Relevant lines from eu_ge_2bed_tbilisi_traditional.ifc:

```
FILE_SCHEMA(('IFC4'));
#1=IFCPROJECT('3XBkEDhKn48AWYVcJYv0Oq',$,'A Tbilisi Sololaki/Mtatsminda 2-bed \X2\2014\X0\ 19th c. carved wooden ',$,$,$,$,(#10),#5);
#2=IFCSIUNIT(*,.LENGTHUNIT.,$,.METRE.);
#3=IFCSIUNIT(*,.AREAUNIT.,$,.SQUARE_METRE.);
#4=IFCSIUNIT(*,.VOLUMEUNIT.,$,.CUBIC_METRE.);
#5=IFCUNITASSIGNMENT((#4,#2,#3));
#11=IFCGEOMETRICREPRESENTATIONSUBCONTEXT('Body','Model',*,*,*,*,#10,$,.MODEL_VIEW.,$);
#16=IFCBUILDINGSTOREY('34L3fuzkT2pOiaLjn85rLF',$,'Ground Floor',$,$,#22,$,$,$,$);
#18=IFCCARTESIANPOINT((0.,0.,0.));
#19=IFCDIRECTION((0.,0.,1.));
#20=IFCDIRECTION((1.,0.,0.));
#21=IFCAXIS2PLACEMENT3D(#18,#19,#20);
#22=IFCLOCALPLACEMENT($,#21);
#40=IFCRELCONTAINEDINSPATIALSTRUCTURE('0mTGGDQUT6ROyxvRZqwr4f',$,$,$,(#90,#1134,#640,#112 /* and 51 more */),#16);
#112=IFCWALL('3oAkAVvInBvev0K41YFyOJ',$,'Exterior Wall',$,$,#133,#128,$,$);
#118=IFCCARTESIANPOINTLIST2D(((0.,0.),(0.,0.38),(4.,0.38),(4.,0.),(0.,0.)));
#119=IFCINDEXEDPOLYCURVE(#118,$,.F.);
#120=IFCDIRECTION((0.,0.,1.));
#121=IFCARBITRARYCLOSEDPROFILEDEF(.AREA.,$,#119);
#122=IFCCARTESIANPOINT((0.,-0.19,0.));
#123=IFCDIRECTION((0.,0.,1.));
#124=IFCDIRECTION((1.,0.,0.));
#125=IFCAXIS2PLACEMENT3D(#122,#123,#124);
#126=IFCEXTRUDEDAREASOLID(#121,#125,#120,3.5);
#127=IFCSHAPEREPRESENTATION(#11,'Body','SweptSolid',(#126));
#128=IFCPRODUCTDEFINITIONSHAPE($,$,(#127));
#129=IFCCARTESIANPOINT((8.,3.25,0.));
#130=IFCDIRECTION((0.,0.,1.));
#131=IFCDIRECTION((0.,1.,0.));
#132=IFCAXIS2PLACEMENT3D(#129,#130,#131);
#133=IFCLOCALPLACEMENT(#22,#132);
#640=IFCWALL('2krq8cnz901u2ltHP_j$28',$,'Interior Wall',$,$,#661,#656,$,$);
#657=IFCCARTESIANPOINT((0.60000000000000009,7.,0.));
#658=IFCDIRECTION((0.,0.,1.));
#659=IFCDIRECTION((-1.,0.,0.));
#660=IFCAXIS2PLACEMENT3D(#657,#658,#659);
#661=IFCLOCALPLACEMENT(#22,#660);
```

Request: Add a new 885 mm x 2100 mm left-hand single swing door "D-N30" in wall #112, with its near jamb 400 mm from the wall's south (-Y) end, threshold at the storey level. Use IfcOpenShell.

```python
import numpy as np
import ifcopenshell
import ifcopenshell.api.feature
import ifcopenshell.api.geometry
import ifcopenshell.api.root
import ifcopenshell.api.spatial
import ifcopenshell.geom
import ifcopenshell.util.element
import ifcopenshell.util.placement
import ifcopenshell.util.representation
import ifcopenshell.util.shape
import ifcopenshell.util.unit

model = ifcopenshell.open("eu_ge_2bed_tbilisi_traditional.ifc")
unit_scale = ifcopenshell.util.unit.calculate_unit_scale(model)
settings = ifcopenshell.geom.settings()


def volume(element):
    """Net volume in cubic metres, openings subtracted."""
    shape = ifcopenshell.geom.create_shape(settings, element)
    return ifcopenshell.util.shape.get_volume(shape.geometry)


wall = model.by_guid("3oAkAVvInBvev0K41YFyOJ")
storey = ifcopenshell.util.element.get_container(wall, ifc_class="IfcBuildingStorey")
context = ifcopenshell.util.representation.get_context(model, "Model", "Body", "MODEL_VIEW")
before = volume(wall)

width, height, from_end, sill = 0.885, 2.1, 0.4, 0.0  # metres

# The wall runs along its own X axis, and the end named is its -X end.
wall_shape = ifcopenshell.geom.create_shape(settings, wall)
x, y, z = ifcopenshell.util.shape.get_vertices(wall_shape.geometry).T
start = x.min() + from_end
face, thickness = float(y.min()), float(y.max() - y.min())
wall_matrix = ifcopenshell.util.placement.get_local_placement(wall.ObjectPlacement)
level = ifcopenshell.util.placement.get_local_placement(storey.ObjectPlacement)[2, 3]


def in_wall(x, y):
    """Placement at x, y metres in the wall's axes, at sill height."""
    matrix = wall_matrix.copy()
    matrix[:, 3] = wall_matrix @ np.array([x / unit_scale, y / unit_scale, 0.0, 1.0])
    matrix[2, 3] = level + sill / unit_scale
    return matrix


# Opening: a box that overshoots both wall faces by 50 mm.
opening = ifcopenshell.api.root.create_entity(model, ifc_class="IfcOpeningElement", predefined_type="OPENING")
box = ifcopenshell.api.geometry.add_wall_representation(
    model, context=context, length=width, height=height, thickness=thickness + 0.1
)
ifcopenshell.api.geometry.assign_representation(model, product=opening, representation=box)
ifcopenshell.api.geometry.edit_object_placement(model, product=opening, matrix=in_wall(start, face - 0.05), is_si=False)
ifcopenshell.api.feature.add_feature(model, feature=opening, element=wall)

door = ifcopenshell.api.root.create_entity(model, ifc_class="IfcDoor", name="D-N30", predefined_type="DOOR")
door.OverallWidth, door.OverallHeight = width / unit_scale, height / unit_scale
door.OperationType = "SINGLE_SWING_LEFT"
body = ifcopenshell.api.geometry.add_door_representation(
    model,
    context=context,
    overall_width=door.OverallWidth,
    overall_height=door.OverallHeight,
    operation_type="SINGLE_SWING_LEFT",
    lining_properties={"LiningDepth": thickness / unit_scale, "ThresholdDepth": thickness / unit_scale},
)
ifcopenshell.api.geometry.assign_representation(model, product=door, representation=body)
ifcopenshell.api.spatial.assign_container(model, products=[door], relating_structure=storey)
ifcopenshell.api.feature.add_filling(model, opening=opening, element=door)

# The lining spans the wall, so the door starts at the wall face.
ifcopenshell.api.geometry.edit_object_placement(model, product=door, matrix=in_wall(start, face), is_si=False)

after = volume(wall)

print(f"wall volume {before:.3f} -> {after:.3f} m3")

model.write("eu_ge_2bed_tbilisi_traditional-out.ifc")
```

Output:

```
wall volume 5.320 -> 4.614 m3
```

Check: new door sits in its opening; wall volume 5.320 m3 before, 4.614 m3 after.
